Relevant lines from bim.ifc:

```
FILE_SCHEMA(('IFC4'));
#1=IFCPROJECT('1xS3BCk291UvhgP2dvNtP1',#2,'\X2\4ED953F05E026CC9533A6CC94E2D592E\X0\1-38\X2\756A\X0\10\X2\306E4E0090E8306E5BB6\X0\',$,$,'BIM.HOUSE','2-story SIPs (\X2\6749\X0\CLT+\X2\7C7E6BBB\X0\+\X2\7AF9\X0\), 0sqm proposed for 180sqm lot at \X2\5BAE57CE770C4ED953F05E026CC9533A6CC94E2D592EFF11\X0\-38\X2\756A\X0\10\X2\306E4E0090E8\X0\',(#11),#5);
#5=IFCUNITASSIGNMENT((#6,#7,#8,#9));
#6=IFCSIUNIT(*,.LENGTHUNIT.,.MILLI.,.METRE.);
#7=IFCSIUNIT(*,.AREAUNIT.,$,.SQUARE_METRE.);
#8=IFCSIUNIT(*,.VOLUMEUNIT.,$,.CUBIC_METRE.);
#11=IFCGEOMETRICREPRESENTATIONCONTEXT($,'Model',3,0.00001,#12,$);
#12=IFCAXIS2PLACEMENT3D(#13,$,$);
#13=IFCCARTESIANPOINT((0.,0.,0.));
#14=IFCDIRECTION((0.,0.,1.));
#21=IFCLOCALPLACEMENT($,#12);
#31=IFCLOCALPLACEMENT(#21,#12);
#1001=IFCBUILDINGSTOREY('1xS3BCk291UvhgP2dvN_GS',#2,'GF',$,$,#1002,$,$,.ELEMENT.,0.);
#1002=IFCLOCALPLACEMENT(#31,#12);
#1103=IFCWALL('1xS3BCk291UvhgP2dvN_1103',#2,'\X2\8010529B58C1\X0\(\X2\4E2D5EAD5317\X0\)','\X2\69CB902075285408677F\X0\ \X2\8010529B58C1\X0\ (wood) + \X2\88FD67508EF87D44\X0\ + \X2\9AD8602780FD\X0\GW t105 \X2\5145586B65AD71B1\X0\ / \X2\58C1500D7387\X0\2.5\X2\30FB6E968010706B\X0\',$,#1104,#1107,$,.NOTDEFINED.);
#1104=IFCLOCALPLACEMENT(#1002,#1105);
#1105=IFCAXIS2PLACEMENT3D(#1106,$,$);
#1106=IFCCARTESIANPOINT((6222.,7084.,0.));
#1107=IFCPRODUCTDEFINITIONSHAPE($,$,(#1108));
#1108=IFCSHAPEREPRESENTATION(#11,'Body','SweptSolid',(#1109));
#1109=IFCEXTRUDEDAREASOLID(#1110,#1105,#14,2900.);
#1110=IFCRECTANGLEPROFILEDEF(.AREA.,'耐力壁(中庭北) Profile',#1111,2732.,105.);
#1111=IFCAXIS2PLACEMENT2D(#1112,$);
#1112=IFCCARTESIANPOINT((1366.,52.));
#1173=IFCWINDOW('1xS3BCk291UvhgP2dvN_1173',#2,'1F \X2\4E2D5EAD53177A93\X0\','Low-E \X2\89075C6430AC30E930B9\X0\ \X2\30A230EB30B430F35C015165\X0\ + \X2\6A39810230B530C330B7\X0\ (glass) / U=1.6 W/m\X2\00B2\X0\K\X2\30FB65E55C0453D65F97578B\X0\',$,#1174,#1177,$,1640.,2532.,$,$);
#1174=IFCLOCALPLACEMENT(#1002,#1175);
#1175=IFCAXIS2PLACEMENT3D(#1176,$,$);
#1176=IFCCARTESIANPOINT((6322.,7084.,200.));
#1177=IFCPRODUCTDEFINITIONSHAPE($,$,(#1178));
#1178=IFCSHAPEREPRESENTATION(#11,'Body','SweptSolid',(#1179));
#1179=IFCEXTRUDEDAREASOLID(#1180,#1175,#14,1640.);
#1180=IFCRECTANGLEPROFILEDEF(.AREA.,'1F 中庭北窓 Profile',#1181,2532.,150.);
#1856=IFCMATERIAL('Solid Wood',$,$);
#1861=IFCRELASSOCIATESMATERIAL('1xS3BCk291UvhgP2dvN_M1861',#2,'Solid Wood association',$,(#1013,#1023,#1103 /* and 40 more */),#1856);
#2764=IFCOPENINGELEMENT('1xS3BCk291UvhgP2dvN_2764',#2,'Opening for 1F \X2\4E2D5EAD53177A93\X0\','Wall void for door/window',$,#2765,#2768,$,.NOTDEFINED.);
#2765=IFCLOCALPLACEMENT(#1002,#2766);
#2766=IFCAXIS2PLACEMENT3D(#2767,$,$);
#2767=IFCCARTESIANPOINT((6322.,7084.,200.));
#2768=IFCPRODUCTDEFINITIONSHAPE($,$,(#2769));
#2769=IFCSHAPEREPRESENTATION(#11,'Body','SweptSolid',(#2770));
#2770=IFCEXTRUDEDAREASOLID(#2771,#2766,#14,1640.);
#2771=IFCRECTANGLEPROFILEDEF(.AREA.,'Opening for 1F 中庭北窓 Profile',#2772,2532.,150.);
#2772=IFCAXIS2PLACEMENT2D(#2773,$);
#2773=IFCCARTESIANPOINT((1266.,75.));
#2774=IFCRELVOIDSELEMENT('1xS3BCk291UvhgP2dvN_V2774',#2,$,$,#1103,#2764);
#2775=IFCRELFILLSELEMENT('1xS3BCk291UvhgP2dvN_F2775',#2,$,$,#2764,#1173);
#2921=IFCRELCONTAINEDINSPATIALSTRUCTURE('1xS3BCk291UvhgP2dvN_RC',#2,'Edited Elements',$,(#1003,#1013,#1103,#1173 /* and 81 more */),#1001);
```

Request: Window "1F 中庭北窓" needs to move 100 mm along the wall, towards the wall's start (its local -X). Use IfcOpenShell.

```python
import ifcopenshell
import ifcopenshell.api.geometry
import ifcopenshell.util.placement
import ifcopenshell.util.unit

model = ifcopenshell.open("bim.ifc")
unit_scale = ifcopenshell.util.unit.calculate_unit_scale(model)

window = model.by_id(1173)
opening = window.FillsVoids[0].RelatingOpeningElement
wall = opening.VoidsElements[0].RelatingBuildingElement

wall_matrix = ifcopenshell.util.placement.get_local_placement(wall.ObjectPlacement)
shift = wall_matrix[:3, 0] * -0.1 / unit_scale
before = ifcopenshell.util.placement.get_local_placement(window.ObjectPlacement)[:3, 3].copy()

# The window is not placed relative to its opening, so move both.
for product in (opening, window):
    matrix = ifcopenshell.util.placement.get_local_placement(product.ObjectPlacement)
    matrix[:3, 3] += shift
    ifcopenshell.api.geometry.edit_object_placement(model, product=product, matrix=matrix, is_si=False)

after = ifcopenshell.util.placement.get_local_placement(window.ObjectPlacement)[:3, 3]
print("window moved by", (after - before).round(3) + 0.0)

model.write("bim_updated.ifc")
```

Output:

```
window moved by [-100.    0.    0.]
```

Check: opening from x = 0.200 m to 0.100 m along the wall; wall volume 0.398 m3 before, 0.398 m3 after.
